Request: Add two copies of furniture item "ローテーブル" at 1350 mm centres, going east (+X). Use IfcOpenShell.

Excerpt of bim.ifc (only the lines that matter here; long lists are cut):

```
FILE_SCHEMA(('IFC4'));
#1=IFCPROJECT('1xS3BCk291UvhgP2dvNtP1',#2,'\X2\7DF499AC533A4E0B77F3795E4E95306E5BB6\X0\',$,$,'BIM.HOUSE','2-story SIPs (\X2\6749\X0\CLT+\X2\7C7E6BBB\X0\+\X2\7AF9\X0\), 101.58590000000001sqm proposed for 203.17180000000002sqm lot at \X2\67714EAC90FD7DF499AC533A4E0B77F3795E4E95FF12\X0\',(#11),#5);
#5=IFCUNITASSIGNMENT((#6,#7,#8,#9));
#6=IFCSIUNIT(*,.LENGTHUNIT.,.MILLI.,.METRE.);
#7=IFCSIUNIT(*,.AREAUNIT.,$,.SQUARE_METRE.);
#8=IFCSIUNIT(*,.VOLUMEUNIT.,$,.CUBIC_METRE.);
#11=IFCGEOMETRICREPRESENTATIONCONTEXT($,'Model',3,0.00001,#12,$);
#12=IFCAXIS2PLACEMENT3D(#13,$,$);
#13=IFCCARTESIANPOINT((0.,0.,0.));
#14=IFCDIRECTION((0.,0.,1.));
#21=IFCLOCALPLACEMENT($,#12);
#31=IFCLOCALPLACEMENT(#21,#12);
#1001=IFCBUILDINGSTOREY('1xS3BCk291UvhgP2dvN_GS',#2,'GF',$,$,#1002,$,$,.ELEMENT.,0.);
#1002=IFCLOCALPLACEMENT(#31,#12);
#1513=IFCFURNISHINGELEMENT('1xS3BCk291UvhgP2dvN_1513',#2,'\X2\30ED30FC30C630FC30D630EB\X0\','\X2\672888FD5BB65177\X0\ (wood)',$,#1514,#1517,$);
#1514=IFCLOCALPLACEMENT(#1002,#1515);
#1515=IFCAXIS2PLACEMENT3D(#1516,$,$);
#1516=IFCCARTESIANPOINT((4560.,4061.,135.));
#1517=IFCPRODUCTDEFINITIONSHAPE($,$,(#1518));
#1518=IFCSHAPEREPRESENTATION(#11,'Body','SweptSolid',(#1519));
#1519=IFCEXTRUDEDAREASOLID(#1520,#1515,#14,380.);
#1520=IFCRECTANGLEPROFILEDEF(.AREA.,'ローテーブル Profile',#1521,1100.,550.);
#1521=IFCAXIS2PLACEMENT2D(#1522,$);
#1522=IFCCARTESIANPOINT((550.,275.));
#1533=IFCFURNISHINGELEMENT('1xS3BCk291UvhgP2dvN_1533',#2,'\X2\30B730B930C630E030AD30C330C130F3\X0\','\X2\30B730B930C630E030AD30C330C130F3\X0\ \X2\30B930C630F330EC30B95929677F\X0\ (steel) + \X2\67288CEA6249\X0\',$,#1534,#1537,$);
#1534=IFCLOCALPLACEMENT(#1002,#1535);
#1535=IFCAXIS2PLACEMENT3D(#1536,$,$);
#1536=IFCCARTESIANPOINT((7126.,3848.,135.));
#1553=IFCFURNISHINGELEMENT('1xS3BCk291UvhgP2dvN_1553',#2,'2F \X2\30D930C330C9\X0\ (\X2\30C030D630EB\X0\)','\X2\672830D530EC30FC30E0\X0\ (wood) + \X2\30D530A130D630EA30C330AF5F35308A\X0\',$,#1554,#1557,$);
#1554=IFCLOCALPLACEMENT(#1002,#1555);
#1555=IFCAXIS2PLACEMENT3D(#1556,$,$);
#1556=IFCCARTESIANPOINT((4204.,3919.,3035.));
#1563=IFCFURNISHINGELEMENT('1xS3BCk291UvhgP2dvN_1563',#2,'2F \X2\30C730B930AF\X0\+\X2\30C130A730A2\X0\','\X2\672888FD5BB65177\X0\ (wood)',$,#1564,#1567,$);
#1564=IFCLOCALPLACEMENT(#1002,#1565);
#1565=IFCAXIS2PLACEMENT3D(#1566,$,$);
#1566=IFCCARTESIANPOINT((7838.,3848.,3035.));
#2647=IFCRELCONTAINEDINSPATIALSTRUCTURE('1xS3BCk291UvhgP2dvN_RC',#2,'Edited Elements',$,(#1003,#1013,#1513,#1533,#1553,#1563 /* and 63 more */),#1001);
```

```python
import numpy as np
import ifcopenshell
import ifcopenshell.api.geometry
import ifcopenshell.api.root
import ifcopenshell.util.element
import ifcopenshell.util.placement
import ifcopenshell.util.unit

model = ifcopenshell.open("bim.ifc")
unit_scale = ifcopenshell.util.unit.calculate_unit_scale(model)


def reuse_history(source, copy):
    """copy_class also copies each property set's owner history, people and application; keep the originals."""
    for rel in copy.IsDefinedBy:
        if rel.is_a("IfcRelDefinesByProperties") and (history := rel.RelatingPropertyDefinition.OwnerHistory):
            rel.RelatingPropertyDefinition.OwnerHistory = source.OwnerHistory
            ifcopenshell.util.element.remove_deep2(model, history)


source = model.by_guid("1xS3BCk291UvhgP2dvN_1513")
base = ifcopenshell.util.placement.get_local_placement(source.ObjectPlacement)
step = np.array([1.0, 0.0, 0.0]) * 1.35 / unit_scale

for i in range(1, 3):
    copy = ifcopenshell.api.root.copy_class(model, product=source)
    copy.Representation = ifcopenshell.util.element.copy_deep(
        model, source.Representation, exclude=["IfcGeometricRepresentationContext", "IfcRepresentationMap"]
    )
    reuse_history(source, copy)
    matrix = base.copy()
    matrix[:3, 3] += i * step
    print("added at", matrix[:3, 3].round(3) + 0.0)
    ifcopenshell.api.geometry.edit_object_placement(model, product=copy, matrix=matrix, is_si=False)

model.write("bim_updated.ifc")
```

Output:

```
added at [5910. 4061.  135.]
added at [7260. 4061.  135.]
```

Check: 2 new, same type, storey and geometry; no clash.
